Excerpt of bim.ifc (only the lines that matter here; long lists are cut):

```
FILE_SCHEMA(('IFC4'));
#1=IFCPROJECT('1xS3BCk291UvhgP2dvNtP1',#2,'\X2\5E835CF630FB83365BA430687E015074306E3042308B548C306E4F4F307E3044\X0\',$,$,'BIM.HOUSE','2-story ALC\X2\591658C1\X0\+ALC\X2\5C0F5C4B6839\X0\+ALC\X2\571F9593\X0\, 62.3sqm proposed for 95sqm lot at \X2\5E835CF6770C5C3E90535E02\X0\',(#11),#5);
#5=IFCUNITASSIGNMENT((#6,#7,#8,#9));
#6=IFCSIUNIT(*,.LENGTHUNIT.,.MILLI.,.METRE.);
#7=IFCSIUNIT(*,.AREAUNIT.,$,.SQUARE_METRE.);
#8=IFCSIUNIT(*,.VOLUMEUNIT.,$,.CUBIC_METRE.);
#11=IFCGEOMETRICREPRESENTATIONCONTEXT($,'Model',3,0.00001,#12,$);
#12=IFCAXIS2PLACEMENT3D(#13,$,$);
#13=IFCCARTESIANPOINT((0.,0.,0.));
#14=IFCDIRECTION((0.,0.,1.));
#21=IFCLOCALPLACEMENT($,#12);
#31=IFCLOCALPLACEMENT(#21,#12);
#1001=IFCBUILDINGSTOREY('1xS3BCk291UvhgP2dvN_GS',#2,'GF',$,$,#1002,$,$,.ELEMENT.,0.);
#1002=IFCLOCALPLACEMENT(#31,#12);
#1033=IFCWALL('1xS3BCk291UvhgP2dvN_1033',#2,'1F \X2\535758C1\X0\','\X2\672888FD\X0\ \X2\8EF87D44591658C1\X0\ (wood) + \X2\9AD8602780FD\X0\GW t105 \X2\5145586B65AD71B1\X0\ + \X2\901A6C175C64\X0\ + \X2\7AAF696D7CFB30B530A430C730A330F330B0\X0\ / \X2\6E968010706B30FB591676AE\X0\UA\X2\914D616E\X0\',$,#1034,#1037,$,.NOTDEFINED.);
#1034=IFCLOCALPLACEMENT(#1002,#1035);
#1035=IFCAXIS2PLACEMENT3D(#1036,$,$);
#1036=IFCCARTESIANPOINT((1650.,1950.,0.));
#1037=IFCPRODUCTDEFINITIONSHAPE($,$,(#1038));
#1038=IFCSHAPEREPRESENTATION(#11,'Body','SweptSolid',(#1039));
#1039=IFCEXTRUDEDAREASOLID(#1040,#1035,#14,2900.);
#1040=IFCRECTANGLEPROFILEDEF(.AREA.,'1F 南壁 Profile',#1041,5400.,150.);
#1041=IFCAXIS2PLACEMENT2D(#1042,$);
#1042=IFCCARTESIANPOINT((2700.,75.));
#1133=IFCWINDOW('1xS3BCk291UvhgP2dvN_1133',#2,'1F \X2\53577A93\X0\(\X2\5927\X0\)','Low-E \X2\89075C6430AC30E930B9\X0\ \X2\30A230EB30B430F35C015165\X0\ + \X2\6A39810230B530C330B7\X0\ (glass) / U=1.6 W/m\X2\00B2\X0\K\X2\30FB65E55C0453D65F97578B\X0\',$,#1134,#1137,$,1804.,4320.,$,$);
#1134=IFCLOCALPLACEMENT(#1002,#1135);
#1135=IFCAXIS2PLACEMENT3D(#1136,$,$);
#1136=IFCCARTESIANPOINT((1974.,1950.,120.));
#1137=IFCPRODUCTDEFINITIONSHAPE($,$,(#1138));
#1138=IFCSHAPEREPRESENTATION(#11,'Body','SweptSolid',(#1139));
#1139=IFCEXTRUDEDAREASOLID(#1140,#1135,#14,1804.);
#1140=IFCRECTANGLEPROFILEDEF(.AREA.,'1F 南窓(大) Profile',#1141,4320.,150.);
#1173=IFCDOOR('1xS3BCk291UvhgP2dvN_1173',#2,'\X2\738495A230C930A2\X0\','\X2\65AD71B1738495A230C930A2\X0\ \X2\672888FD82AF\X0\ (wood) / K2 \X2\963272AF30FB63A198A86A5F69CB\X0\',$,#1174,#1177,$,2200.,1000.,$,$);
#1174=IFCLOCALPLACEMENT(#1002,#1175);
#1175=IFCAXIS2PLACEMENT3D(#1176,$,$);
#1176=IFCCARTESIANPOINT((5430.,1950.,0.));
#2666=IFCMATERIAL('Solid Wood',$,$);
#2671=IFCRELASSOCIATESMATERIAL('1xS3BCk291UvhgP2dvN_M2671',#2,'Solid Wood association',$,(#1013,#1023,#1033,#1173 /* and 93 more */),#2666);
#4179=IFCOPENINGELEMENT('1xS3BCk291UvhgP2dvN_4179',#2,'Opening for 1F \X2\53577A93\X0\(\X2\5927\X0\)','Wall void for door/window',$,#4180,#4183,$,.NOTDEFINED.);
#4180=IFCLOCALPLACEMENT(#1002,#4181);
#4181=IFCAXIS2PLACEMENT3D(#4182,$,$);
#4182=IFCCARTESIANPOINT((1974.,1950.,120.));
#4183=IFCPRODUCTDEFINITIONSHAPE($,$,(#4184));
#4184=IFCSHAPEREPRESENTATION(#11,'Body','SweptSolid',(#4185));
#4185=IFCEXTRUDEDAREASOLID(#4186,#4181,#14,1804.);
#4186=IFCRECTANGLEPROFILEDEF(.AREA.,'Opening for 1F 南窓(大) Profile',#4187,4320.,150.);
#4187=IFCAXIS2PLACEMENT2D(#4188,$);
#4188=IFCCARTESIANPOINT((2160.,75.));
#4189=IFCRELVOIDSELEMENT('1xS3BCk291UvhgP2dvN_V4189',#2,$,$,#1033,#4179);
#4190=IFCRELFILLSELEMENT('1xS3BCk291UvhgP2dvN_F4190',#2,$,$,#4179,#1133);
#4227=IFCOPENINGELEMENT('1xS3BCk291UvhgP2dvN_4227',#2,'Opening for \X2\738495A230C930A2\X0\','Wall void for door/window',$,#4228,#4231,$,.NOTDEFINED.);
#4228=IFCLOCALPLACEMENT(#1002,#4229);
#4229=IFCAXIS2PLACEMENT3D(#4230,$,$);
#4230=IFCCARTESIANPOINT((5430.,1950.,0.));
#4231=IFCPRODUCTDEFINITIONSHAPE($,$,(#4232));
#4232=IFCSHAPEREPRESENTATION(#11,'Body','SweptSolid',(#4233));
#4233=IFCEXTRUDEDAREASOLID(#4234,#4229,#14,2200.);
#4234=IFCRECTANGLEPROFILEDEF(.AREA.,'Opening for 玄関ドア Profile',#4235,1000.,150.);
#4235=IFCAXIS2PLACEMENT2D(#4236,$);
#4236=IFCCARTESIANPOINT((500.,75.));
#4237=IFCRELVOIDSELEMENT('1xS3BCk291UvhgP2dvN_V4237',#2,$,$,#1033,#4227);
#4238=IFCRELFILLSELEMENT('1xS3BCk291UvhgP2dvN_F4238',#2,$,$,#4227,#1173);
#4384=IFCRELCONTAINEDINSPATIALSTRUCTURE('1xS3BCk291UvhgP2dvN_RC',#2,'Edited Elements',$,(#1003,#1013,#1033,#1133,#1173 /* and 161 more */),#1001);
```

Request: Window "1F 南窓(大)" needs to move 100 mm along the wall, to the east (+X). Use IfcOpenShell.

```python
import ifcopenshell
import ifcopenshell.api.geometry
import ifcopenshell.util.placement
import ifcopenshell.util.unit

model = ifcopenshell.open("bim.ifc")
unit_scale = ifcopenshell.util.unit.calculate_unit_scale(model)

window = model.by_guid("1xS3BCk291UvhgP2dvN_1133")
opening = window.FillsVoids[0].RelatingOpeningElement
wall = opening.VoidsElements[0].RelatingBuildingElement

wall_matrix = ifcopenshell.util.placement.get_local_placement(wall.ObjectPlacement)
shift = wall_matrix[:3, 0] * 0.1 / unit_scale
before = ifcopenshell.util.placement.get_local_placement(window.ObjectPlacement)[:3, 3].copy()

# The window is not placed relative to its opening, so move both.
for product in (opening, window):
    matrix = ifcopenshell.util.placement.get_local_placement(product.ObjectPlacement)
    matrix[:3, 3] += shift
    ifcopenshell.api.geometry.edit_object_placement(model, product=product, matrix=matrix, is_si=False)

after = ifcopenshell.util.placement.get_local_placement(window.ObjectPlacement)[:3, 3]
print("window moved by", (after - before).round(3) + 0.0)

model.write("bim_v2.ifc")
```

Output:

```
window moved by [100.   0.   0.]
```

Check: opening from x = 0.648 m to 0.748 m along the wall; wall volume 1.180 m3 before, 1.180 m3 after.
